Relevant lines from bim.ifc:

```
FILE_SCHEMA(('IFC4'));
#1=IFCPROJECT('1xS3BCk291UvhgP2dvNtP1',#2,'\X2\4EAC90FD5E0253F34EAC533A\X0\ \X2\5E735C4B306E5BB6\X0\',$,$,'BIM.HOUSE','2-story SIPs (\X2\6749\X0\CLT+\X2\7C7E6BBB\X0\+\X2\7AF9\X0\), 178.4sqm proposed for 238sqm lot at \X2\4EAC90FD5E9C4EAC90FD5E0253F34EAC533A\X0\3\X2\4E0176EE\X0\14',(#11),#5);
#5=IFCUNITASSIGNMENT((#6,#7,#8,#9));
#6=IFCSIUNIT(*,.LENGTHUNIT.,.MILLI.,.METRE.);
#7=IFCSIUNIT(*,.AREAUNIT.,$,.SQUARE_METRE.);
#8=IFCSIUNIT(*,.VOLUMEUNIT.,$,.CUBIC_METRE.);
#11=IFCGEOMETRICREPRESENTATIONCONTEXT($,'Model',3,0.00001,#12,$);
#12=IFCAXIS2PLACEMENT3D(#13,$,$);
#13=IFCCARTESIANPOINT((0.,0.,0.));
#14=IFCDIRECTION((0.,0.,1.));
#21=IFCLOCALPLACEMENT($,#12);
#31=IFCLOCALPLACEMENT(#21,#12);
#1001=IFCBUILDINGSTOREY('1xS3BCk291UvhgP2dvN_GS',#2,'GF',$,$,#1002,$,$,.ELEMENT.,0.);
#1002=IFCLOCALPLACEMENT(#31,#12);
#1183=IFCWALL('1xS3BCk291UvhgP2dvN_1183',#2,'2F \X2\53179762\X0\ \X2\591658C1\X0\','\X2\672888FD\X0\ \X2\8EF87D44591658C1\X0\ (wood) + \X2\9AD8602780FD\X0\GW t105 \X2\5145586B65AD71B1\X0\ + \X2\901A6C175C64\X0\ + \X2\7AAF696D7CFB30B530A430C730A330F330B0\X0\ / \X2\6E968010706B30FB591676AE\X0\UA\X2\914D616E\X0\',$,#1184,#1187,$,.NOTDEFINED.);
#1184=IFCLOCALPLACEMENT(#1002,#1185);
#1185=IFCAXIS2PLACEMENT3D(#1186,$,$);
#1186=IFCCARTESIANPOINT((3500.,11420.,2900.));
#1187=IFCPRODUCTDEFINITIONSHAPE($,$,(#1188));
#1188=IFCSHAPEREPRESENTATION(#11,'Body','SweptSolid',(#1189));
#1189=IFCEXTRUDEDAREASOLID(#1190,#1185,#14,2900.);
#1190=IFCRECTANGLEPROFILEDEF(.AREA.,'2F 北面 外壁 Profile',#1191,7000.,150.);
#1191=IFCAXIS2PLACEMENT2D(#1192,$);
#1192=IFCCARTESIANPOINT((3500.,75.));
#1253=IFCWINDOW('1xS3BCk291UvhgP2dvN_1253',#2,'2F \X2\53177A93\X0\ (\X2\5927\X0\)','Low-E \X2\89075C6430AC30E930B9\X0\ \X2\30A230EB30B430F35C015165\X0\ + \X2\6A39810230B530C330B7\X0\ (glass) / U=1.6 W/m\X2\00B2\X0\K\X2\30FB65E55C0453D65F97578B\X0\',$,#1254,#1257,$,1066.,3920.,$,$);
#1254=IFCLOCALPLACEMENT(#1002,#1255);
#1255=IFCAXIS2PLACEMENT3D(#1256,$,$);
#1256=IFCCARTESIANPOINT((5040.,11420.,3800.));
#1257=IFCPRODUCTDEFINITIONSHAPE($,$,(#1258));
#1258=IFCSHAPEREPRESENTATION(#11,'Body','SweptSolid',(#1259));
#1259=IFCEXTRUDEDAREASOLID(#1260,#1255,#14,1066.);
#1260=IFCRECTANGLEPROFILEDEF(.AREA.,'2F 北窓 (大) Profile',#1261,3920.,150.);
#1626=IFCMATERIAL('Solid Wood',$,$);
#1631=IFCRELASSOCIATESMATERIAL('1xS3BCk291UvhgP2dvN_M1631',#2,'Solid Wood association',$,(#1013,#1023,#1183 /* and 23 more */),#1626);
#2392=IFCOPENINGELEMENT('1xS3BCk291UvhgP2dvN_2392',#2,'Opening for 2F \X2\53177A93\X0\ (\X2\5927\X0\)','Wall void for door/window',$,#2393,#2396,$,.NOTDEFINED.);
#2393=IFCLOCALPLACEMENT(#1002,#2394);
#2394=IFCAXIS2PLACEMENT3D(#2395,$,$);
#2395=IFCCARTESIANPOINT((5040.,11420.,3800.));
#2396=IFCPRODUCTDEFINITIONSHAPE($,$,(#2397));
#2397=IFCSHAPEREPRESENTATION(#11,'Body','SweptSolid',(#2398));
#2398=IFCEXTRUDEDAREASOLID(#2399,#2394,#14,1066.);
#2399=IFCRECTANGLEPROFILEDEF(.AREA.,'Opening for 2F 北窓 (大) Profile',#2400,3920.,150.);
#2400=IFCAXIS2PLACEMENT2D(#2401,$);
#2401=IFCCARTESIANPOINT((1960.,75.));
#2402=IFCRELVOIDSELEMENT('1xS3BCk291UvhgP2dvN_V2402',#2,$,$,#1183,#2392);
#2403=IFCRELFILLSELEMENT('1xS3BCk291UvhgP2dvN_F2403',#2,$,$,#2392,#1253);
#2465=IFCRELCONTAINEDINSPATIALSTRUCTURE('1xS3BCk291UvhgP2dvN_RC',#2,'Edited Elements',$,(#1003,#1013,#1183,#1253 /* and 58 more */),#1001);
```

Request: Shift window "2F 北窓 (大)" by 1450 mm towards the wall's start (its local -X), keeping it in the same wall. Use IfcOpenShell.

```python
import ifcopenshell
import ifcopenshell.api.geometry
import ifcopenshell.util.placement
import ifcopenshell.util.unit

model = ifcopenshell.open("bim.ifc")
unit_scale = ifcopenshell.util.unit.calculate_unit_scale(model)

window = model.by_guid("1xS3BCk291UvhgP2dvN_1253")
opening = window.FillsVoids[0].RelatingOpeningElement
wall = opening.VoidsElements[0].RelatingBuildingElement

wall_matrix = ifcopenshell.util.placement.get_local_placement(wall.ObjectPlacement)
shift = wall_matrix[:3, 0] * -1.45 / unit_scale
before = ifcopenshell.util.placement.get_local_placement(window.ObjectPlacement)[:3, 3].copy()

# The window is not placed relative to its opening, so move both.
for product in (opening, window):
    matrix = ifcopenshell.util.placement.get_local_placement(product.ObjectPlacement)
    matrix[:3, 3] += shift
    ifcopenshell.api.geometry.edit_object_placement(model, product=product, matrix=matrix, is_si=False)

after = ifcopenshell.util.placement.get_local_placement(window.ObjectPlacement)[:3, 3]
print("window moved by", (after - before).round(3) + 0.0)

model.write("bim_rev.ifc")
```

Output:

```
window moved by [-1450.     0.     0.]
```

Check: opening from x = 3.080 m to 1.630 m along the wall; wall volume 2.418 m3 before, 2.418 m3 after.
